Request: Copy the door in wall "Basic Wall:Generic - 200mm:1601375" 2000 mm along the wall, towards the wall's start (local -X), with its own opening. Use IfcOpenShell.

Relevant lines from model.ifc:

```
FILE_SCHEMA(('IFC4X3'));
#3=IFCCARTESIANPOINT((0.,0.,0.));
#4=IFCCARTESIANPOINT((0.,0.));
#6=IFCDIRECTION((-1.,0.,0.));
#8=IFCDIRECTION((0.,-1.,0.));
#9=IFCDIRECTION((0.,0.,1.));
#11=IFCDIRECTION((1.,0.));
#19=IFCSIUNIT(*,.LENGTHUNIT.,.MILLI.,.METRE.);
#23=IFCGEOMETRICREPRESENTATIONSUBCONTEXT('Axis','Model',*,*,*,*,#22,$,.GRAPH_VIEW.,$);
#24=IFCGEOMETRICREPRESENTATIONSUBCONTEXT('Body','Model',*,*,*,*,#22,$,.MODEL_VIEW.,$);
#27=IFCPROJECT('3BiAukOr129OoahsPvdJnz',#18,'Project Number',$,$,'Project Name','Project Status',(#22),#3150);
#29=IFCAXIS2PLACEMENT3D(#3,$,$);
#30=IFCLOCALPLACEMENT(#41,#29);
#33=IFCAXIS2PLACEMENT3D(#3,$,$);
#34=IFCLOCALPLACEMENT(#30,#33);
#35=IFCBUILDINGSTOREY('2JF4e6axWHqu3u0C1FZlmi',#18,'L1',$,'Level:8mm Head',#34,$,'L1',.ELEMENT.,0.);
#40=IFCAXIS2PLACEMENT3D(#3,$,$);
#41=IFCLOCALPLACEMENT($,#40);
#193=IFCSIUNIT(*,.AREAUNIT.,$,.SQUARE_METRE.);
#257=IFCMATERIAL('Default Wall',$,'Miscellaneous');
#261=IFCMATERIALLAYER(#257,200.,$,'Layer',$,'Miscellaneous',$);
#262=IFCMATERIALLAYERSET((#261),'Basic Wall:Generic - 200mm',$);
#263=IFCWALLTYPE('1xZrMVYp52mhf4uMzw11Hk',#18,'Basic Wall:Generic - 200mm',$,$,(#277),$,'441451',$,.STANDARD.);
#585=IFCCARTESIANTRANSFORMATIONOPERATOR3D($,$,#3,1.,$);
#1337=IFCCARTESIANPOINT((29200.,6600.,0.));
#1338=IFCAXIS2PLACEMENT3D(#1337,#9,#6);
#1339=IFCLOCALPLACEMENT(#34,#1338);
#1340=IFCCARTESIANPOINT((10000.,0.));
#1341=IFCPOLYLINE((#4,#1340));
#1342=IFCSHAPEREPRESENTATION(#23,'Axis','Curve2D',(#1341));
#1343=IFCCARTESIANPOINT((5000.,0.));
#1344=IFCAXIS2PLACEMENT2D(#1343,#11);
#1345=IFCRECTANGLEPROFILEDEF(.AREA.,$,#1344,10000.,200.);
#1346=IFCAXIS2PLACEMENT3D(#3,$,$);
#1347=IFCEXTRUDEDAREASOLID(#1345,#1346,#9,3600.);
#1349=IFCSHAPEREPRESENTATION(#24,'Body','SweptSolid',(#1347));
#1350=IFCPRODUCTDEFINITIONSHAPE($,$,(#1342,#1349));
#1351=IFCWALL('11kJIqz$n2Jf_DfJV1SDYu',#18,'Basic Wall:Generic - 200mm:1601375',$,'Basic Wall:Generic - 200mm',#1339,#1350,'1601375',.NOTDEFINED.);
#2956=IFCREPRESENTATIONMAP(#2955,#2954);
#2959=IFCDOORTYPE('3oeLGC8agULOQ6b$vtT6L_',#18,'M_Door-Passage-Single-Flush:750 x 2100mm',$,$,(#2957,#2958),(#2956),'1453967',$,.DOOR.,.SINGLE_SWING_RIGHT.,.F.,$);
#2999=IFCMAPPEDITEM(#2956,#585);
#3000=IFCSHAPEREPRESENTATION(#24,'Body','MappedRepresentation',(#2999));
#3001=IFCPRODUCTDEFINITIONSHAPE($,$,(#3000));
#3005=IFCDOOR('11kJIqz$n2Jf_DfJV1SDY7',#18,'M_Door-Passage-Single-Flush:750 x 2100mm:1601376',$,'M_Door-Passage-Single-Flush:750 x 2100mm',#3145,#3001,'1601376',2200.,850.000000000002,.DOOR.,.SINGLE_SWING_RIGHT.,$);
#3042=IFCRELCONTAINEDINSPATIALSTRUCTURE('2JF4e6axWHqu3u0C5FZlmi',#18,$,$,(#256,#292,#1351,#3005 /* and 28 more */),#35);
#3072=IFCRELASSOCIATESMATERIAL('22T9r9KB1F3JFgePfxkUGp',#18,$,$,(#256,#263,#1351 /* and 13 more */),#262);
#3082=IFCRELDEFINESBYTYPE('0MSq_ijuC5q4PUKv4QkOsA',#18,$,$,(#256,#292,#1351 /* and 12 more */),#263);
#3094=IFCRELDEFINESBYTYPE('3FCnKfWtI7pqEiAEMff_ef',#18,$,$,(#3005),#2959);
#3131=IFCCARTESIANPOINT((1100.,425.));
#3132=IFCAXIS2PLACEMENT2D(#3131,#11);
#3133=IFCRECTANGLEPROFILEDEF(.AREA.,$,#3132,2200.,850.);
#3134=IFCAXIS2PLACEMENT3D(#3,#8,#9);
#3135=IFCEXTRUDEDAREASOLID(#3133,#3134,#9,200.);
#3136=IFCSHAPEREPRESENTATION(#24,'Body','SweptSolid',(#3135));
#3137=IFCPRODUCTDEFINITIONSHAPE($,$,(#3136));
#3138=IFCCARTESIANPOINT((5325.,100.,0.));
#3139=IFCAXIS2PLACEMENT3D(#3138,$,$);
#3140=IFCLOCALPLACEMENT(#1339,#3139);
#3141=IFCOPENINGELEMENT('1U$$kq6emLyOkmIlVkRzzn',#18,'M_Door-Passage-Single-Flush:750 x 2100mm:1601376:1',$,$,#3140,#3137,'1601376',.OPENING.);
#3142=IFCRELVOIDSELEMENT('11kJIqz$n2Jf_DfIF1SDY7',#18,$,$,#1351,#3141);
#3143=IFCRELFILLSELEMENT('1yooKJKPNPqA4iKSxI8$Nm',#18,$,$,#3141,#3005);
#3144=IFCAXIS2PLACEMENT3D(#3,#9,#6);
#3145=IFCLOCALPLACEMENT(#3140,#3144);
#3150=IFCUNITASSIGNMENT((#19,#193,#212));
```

```python
import ifcopenshell
import ifcopenshell.api.feature
import ifcopenshell.api.geometry
import ifcopenshell.api.root
import ifcopenshell.geom
import ifcopenshell.util.element
import ifcopenshell.util.placement
import ifcopenshell.util.shape
import ifcopenshell.util.unit

model = ifcopenshell.open("model.ifc")
unit_scale = ifcopenshell.util.unit.calculate_unit_scale(model)
settings = ifcopenshell.geom.settings()


def volume(element):
    """Net volume in cubic metres, openings subtracted."""
    shape = ifcopenshell.geom.create_shape(settings, element)
    return ifcopenshell.util.shape.get_volume(shape.geometry)


def reuse_history(source, copy):
    """copy_class also copies each property set's owner history, people and application; keep the originals."""
    for rel in copy.IsDefinedBy:
        if rel.is_a("IfcRelDefinesByProperties") and (history := rel.RelatingPropertyDefinition.OwnerHistory):
            rel.RelatingPropertyDefinition.OwnerHistory = source.OwnerHistory
            ifcopenshell.util.element.remove_deep2(model, history)


door = model.by_guid("11kJIqz$n2Jf_DfJV1SDY7")
opening = door.FillsVoids[0].RelatingOpeningElement
wall = opening.VoidsElements[0].RelatingBuildingElement
before = volume(wall)
shift = ifcopenshell.util.placement.get_local_placement(wall.ObjectPlacement)[:3, 0] * -2 / unit_scale

# copy_class copies the void relationship, type, container and properties, but no geometry.
new_opening = ifcopenshell.api.root.copy_class(model, product=opening)
new_opening.Representation = ifcopenshell.util.element.copy_deep(
    model, opening.Representation, exclude=["IfcGeometricRepresentationContext", "IfcRepresentationMap"]
)
new_opening.Name = "M_Door-Passage-Single-Flush:750 x 2100mm"
new_opening.Tag = None
new_door = ifcopenshell.api.root.copy_class(model, product=door)
new_door.Representation = ifcopenshell.util.element.copy_deep(
    model, door.Representation, exclude=["IfcGeometricRepresentationContext", "IfcRepresentationMap"]
)
new_door.Name = "M_Door-Passage-Single-Flush:750 x 2100mm"
new_door.Tag = None
reuse_history(door, new_door)
ifcopenshell.api.feature.add_filling(model, opening=new_opening, element=new_door)

for old, new in ((opening, new_opening), (door, new_door)):
    matrix = ifcopenshell.util.placement.get_local_placement(old.ObjectPlacement)
    matrix[:3, 3] += shift
    ifcopenshell.api.geometry.edit_object_placement(model, product=new, matrix=matrix, is_si=False)

after = volume(wall)

print(f"wall volume {before:.3f} -> {after:.3f} m3")

model.write("model_updated.ifc")
```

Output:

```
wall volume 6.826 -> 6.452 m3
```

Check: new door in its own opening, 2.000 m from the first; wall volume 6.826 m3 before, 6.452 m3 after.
